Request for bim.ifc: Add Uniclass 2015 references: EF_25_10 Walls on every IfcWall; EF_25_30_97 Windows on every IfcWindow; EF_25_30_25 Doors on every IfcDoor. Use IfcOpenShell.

First a look at what the model holds.

```python
import ifcopenshell

model = ifcopenshell.open("bim.ifc")
print(model.schema)
print("classifications:", [c.Name for c in model.by_type("IfcClassification")])
for ifc_class in ("IfcDoor", "IfcRoof", "IfcStair", "IfcWall", "IfcWindow"):
    print(ifc_class, len(model.by_type(ifc_class)))
```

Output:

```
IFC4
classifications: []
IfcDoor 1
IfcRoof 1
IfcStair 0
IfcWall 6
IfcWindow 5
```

```python
import ifcopenshell
import ifcopenshell.api.classification

model = ifcopenshell.open("bim.ifc")

system = ifcopenshell.api.classification.add_classification(model, classification="Uniclass 2015")

codes = {
    "IfcWall": ("EF_25_10", "Walls"),
    "IfcWindow": ("EF_25_30_97", "Windows"),
    "IfcDoor": ("EF_25_30_25", "Doors"),
}
for ifc_class, (code, name) in codes.items():
    products = model.by_type(ifc_class)
    ifcopenshell.api.classification.add_reference(
        model, products=products, classification=system, identification=code, name=name
    )
    print(code, len(products))

model.write("bim_updated.ifc")
```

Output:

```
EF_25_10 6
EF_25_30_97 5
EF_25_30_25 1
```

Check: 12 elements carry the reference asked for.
